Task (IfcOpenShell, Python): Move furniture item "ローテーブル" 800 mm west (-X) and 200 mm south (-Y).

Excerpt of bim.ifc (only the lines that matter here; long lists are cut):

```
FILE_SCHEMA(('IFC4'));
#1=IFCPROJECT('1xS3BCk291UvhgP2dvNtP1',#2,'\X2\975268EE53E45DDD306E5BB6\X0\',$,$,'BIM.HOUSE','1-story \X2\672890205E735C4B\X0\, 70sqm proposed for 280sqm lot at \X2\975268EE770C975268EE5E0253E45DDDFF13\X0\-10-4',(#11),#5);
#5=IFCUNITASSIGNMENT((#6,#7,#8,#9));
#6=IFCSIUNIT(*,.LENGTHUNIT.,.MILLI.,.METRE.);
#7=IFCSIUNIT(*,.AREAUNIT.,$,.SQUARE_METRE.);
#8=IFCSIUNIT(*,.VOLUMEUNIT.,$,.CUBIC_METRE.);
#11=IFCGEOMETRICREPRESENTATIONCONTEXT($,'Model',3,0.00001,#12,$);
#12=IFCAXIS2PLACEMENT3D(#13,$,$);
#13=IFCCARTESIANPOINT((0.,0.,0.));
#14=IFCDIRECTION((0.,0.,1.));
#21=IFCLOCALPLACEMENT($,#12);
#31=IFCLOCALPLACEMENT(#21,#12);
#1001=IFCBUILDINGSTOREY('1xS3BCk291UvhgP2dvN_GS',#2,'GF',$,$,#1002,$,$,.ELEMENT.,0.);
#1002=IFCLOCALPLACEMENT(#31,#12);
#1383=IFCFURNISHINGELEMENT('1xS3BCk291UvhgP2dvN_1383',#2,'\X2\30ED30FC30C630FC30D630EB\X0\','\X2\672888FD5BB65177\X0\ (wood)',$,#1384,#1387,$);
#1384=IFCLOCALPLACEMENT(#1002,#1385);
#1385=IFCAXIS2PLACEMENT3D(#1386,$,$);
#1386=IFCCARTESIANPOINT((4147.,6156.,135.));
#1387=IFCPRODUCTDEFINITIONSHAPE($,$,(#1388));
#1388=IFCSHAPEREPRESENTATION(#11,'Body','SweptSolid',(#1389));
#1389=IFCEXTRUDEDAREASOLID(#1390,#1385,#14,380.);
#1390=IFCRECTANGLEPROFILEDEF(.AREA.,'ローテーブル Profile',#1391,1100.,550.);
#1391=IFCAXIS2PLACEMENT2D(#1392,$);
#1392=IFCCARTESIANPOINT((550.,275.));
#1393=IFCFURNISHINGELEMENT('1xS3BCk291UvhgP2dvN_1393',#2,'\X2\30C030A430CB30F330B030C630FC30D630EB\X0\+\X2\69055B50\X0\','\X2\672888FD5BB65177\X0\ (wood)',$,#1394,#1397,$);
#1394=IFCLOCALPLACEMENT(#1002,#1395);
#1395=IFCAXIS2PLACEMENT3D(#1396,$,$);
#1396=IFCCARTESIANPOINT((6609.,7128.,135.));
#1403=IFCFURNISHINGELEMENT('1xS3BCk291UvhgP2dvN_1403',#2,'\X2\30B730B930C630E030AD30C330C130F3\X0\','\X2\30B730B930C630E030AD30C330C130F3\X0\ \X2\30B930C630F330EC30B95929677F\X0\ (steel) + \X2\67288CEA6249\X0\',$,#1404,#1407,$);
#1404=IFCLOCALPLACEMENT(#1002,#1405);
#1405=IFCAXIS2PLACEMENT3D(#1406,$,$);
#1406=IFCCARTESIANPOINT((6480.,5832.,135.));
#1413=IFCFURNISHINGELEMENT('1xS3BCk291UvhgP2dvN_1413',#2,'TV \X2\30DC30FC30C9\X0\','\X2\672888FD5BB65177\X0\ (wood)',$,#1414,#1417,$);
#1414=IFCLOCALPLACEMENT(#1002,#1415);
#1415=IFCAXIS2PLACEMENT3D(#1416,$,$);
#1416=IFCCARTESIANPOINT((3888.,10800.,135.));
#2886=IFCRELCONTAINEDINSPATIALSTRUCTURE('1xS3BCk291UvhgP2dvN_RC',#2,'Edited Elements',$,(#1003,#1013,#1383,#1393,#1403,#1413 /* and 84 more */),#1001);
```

```python
import ifcopenshell
import ifcopenshell.api.geometry
import ifcopenshell.util.placement
import ifcopenshell.util.unit

model = ifcopenshell.open("bim.ifc")
unit_scale = ifcopenshell.util.unit.calculate_unit_scale(model)

item = model.by_guid("1xS3BCk291UvhgP2dvN_1383")
matrix = ifcopenshell.util.placement.get_local_placement(item.ObjectPlacement)
matrix[0, 3] -= 0.8 / unit_scale
matrix[1, 3] -= 0.2 / unit_scale
ifcopenshell.api.geometry.edit_object_placement(model, product=item, matrix=matrix, is_si=False)

print(ifcopenshell.util.placement.get_local_placement(item.ObjectPlacement).round(3) + 0.0)

model.write("bim_updated.ifc")
```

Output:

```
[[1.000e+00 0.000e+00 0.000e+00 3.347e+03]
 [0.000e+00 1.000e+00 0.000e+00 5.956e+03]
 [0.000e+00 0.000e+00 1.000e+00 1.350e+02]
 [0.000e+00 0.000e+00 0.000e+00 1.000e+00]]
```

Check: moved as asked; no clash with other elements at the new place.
